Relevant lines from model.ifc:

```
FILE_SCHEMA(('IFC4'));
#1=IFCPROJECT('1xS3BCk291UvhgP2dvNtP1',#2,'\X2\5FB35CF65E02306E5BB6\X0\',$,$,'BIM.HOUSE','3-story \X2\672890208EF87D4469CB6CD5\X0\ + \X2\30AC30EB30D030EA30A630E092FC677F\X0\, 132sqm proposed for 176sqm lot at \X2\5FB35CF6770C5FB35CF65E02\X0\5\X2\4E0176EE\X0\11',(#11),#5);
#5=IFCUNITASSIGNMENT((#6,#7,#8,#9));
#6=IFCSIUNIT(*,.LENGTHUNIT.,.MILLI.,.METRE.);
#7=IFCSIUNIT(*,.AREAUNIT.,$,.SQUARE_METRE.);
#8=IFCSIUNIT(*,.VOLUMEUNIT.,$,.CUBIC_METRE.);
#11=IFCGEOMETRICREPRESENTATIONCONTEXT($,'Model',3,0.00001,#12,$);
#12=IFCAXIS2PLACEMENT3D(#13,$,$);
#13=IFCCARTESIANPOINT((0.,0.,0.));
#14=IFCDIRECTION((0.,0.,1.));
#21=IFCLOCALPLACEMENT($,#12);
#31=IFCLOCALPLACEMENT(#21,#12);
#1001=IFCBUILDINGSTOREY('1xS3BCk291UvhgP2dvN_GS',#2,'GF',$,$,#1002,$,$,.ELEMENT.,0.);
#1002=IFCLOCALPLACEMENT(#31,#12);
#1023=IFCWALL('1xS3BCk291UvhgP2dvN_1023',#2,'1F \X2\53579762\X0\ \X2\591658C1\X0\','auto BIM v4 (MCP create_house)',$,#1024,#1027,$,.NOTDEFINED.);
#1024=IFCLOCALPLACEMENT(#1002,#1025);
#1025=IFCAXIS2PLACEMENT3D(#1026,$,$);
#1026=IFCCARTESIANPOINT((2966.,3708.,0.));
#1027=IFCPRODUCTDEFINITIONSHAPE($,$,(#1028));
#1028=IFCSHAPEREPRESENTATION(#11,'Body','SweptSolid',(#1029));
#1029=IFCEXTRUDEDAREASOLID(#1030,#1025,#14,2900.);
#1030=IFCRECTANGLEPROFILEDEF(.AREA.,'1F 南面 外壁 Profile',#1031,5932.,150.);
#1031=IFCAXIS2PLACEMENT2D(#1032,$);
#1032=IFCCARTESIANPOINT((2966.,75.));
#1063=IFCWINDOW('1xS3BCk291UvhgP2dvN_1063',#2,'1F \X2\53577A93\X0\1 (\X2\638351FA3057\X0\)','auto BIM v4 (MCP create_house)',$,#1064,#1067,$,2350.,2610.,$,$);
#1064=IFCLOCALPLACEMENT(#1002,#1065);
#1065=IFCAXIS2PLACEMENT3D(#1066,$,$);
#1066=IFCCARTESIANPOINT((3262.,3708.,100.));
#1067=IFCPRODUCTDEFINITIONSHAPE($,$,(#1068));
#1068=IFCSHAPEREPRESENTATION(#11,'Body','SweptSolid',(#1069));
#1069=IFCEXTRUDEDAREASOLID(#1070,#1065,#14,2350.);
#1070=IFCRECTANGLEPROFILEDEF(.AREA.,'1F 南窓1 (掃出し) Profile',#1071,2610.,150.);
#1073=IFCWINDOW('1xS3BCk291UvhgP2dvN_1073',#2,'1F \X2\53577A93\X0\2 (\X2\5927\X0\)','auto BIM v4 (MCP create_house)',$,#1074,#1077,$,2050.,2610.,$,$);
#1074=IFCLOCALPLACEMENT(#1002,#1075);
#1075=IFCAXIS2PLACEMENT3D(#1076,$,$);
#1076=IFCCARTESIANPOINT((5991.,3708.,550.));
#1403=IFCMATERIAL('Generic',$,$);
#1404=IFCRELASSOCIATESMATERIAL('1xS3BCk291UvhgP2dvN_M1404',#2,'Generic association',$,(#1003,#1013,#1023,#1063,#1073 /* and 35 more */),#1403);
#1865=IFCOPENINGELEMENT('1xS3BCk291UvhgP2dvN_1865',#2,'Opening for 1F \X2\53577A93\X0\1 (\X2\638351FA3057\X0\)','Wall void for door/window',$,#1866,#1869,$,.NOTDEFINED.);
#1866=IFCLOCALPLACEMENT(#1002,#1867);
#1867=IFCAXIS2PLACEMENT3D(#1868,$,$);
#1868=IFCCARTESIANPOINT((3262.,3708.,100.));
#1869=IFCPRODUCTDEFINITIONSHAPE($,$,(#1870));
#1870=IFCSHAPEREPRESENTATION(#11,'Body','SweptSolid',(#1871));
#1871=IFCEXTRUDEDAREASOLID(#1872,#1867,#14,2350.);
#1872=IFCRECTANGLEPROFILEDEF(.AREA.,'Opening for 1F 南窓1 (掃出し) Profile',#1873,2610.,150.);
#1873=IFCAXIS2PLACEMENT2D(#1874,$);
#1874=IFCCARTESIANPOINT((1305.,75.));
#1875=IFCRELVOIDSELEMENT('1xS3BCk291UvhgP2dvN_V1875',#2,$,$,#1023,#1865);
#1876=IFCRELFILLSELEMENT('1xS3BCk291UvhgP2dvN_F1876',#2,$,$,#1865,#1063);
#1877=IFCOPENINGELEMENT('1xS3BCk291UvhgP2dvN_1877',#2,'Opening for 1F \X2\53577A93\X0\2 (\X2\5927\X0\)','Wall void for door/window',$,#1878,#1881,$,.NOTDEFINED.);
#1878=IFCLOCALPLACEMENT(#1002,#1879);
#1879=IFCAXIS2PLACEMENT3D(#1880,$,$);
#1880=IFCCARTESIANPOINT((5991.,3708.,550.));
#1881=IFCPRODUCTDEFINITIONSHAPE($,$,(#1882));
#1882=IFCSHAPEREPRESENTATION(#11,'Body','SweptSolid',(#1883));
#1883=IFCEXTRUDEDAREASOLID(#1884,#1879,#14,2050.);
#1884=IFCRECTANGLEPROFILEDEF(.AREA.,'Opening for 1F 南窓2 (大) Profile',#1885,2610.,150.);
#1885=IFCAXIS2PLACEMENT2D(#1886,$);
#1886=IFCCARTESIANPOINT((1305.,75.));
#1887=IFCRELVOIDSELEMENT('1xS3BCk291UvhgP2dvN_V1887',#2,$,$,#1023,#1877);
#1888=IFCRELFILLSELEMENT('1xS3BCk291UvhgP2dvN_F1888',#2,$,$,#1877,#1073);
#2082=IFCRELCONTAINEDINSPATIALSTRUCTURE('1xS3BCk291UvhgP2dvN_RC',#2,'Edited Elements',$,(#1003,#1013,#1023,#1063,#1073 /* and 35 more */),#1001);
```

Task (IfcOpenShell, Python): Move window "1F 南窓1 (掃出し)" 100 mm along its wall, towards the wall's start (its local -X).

```python
import ifcopenshell
import ifcopenshell.api.geometry
import ifcopenshell.util.placement
import ifcopenshell.util.unit

model = ifcopenshell.open("model.ifc")
unit_scale = ifcopenshell.util.unit.calculate_unit_scale(model)

window = model.by_guid("1xS3BCk291UvhgP2dvN_1063")
opening = window.FillsVoids[0].RelatingOpeningElement
wall = opening.VoidsElements[0].RelatingBuildingElement

wall_matrix = ifcopenshell.util.placement.get_local_placement(wall.ObjectPlacement)
shift = wall_matrix[:3, 0] * -0.1 / unit_scale
before = ifcopenshell.util.placement.get_local_placement(window.ObjectPlacement)[:3, 3].copy()

# The window is not placed relative to its opening, so move both.
for product in (opening, window):
    matrix = ifcopenshell.util.placement.get_local_placement(product.ObjectPlacement)
    matrix[:3, 3] += shift
    ifcopenshell.api.geometry.edit_object_placement(model, product=product, matrix=matrix, is_si=False)

after = ifcopenshell.util.placement.get_local_placement(window.ObjectPlacement)[:3, 3]
print("window moved by", (after - before).round(3) + 0.0)

model.write("model_updated.ifc")
```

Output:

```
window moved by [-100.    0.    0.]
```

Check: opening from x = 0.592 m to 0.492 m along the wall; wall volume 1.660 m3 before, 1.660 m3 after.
